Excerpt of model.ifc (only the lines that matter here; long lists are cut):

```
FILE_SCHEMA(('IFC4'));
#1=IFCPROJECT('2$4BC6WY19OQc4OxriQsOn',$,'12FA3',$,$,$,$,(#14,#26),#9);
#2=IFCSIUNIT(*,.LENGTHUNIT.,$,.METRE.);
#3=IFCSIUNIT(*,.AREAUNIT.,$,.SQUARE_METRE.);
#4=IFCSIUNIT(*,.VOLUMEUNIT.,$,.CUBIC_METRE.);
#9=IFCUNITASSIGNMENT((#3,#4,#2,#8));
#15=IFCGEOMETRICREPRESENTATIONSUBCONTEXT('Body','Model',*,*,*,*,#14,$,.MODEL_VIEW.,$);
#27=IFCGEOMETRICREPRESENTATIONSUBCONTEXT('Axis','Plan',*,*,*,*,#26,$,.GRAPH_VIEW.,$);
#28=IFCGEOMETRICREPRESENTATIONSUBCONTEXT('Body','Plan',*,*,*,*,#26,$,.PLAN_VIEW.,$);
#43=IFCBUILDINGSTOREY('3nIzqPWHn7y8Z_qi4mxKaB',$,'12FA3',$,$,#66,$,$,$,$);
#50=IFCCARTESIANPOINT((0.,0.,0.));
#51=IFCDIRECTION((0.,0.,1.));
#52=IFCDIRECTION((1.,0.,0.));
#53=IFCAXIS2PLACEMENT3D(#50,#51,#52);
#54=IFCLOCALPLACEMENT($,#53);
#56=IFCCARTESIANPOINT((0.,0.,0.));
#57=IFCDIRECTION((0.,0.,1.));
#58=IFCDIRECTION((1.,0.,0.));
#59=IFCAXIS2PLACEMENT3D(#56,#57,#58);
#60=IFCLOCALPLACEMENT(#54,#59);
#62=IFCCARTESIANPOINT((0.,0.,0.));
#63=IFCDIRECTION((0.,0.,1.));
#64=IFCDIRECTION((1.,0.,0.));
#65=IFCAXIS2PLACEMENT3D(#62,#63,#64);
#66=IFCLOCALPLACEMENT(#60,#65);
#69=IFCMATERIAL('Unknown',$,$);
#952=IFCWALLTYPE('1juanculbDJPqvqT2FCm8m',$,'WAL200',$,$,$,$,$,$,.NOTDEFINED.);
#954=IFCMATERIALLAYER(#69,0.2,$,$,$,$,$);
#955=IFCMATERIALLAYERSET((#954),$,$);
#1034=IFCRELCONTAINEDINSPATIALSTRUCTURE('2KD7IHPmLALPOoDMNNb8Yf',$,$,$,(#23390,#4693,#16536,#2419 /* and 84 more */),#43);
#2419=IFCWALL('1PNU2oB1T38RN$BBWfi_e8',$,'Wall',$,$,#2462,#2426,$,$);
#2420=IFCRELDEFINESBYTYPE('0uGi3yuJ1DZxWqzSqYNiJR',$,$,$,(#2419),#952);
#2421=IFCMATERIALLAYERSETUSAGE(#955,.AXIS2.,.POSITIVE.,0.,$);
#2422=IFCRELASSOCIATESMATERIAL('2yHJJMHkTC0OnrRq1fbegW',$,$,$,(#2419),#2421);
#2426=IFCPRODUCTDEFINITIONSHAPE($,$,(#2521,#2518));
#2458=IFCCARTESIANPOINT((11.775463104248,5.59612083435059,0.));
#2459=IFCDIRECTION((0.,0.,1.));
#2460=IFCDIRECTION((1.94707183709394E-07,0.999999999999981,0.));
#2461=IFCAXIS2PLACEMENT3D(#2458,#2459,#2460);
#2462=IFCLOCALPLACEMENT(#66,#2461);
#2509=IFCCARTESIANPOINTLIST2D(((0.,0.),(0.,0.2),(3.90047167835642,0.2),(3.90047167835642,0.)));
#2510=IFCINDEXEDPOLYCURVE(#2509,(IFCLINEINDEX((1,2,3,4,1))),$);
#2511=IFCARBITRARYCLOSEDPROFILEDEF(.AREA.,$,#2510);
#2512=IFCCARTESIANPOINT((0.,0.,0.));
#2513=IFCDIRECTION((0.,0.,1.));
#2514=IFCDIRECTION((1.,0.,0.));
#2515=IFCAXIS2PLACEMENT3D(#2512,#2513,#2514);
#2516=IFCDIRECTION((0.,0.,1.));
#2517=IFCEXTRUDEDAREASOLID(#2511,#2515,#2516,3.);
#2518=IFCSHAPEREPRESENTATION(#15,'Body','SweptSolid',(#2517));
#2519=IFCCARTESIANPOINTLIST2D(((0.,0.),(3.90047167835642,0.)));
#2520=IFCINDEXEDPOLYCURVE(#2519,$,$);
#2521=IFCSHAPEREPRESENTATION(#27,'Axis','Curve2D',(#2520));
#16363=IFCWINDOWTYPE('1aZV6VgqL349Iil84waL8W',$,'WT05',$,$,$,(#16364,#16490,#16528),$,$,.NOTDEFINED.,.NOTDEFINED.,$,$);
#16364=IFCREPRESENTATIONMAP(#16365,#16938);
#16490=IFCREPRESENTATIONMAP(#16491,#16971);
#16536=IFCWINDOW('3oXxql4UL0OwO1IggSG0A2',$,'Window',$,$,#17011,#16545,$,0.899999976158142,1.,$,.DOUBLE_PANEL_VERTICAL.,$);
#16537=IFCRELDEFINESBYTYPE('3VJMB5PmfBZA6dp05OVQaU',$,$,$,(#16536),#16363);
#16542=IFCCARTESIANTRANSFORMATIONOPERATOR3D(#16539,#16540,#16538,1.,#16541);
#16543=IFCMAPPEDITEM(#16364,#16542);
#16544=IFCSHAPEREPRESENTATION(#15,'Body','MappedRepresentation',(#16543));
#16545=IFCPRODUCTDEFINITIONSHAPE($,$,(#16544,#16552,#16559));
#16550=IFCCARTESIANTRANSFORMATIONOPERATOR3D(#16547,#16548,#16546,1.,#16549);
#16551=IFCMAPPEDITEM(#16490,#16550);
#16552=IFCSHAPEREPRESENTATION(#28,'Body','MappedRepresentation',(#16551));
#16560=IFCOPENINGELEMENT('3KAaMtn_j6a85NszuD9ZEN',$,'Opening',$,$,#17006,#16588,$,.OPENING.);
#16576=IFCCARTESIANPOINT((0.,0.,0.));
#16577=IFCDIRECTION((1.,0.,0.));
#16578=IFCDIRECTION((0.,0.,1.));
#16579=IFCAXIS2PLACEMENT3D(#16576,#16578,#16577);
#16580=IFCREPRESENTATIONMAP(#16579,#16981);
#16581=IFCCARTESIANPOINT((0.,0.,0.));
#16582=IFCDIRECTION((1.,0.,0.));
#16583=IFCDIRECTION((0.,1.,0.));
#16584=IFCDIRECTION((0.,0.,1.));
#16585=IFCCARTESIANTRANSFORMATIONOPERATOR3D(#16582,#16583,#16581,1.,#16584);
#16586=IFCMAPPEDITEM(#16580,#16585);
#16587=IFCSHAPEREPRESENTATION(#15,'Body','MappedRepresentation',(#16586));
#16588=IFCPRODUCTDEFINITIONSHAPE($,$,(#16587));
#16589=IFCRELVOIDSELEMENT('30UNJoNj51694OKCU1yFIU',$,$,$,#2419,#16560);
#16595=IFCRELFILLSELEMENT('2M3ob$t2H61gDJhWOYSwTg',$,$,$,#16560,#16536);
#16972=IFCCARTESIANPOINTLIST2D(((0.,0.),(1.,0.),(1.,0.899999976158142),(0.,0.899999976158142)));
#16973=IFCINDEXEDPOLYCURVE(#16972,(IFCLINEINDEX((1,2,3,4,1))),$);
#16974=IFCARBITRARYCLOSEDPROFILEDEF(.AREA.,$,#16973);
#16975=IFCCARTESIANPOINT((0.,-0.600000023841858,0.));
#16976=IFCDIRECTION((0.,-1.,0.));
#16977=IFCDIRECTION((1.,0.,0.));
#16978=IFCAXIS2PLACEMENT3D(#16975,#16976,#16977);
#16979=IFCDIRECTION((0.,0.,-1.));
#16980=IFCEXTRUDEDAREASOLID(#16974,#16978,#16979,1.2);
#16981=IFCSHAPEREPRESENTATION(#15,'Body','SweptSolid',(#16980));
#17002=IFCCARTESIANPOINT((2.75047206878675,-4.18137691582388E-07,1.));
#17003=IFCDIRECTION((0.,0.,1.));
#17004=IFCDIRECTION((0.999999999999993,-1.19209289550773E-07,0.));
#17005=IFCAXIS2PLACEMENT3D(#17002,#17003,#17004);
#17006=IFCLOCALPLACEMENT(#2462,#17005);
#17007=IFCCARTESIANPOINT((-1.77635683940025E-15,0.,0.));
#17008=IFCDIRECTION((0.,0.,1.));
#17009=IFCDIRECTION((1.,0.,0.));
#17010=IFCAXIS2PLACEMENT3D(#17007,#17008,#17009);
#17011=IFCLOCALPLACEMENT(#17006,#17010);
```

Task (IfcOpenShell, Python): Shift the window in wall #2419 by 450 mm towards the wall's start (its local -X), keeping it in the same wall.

```python
import ifcopenshell
import ifcopenshell.api.geometry
import ifcopenshell.util.placement

model = ifcopenshell.open("model.ifc")

window = model.by_guid("3oXxql4UL0OwO1IggSG0A2")
opening = window.FillsVoids[0].RelatingOpeningElement
wall = opening.VoidsElements[0].RelatingBuildingElement

wall_matrix = ifcopenshell.util.placement.get_local_placement(wall.ObjectPlacement)
shift = wall_matrix[:3, 0] * -0.45
before = ifcopenshell.util.placement.get_local_placement(window.ObjectPlacement)[:3, 3].copy()

# The window is placed relative to its opening, so it follows when the opening moves.
matrix = ifcopenshell.util.placement.get_local_placement(opening.ObjectPlacement)
matrix[:3, 3] += shift
ifcopenshell.api.geometry.edit_object_placement(
    model, product=opening, matrix=matrix, is_si=False, should_transform_children=True
)

after = ifcopenshell.util.placement.get_local_placement(window.ObjectPlacement)[:3, 3]
print("window moved by", (after - before).round(3) + 0.0)

model.write("model_edited.ifc")
```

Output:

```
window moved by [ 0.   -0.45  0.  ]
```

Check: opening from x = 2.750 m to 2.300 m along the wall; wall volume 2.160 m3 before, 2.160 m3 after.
